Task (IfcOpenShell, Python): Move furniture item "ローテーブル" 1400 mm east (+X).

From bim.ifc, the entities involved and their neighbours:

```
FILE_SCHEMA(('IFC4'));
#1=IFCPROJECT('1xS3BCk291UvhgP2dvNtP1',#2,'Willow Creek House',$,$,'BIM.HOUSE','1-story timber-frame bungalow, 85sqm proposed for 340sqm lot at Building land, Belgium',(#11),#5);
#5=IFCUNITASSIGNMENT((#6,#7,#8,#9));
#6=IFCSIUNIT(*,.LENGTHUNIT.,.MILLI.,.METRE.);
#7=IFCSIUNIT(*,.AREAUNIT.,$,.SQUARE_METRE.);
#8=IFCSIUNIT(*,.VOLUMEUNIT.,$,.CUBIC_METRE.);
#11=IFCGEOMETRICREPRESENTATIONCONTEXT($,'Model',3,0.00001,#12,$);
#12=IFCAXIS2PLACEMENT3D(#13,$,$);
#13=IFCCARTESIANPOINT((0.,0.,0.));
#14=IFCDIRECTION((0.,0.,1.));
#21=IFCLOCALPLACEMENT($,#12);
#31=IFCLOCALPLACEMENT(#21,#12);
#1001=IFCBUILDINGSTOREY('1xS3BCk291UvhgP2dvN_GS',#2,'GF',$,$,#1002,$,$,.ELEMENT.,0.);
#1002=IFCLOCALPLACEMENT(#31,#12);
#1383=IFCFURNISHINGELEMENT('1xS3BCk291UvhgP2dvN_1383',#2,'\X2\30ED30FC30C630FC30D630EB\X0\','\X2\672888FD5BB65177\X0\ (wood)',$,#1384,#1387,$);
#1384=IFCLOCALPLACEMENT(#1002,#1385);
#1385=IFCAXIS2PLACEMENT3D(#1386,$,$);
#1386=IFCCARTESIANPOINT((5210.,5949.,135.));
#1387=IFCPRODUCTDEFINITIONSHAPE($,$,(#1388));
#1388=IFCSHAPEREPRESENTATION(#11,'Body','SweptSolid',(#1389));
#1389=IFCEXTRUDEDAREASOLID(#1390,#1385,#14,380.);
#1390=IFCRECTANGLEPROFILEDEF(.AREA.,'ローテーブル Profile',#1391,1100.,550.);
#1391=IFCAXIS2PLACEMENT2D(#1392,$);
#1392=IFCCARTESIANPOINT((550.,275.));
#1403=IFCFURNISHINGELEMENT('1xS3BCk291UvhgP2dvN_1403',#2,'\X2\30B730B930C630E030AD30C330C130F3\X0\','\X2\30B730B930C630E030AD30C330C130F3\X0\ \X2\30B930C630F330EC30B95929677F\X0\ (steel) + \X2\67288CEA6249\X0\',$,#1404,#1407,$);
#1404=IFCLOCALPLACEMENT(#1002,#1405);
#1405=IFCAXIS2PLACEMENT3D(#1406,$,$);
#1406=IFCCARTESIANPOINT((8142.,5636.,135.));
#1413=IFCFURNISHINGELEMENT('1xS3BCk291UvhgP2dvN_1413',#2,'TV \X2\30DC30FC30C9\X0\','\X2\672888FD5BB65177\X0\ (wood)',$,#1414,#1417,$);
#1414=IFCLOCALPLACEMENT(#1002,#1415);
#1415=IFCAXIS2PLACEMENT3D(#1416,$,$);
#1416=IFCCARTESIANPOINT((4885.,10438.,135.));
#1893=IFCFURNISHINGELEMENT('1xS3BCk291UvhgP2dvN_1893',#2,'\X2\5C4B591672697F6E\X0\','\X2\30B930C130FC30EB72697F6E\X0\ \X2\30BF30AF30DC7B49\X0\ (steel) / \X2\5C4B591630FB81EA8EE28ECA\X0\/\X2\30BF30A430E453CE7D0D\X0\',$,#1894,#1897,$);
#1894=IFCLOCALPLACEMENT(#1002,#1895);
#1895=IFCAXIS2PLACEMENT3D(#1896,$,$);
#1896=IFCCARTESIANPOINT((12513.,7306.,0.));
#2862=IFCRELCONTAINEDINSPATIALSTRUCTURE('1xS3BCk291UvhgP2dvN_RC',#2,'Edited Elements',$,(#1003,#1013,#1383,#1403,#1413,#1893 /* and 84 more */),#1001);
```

```python
import ifcopenshell
import ifcopenshell.api.geometry
import ifcopenshell.util.placement
import ifcopenshell.util.unit

model = ifcopenshell.open("bim.ifc")
unit_scale = ifcopenshell.util.unit.calculate_unit_scale(model)

item = model.by_guid("1xS3BCk291UvhgP2dvN_1383")
matrix = ifcopenshell.util.placement.get_local_placement(item.ObjectPlacement)
matrix[0, 3] += 1.4 / unit_scale
ifcopenshell.api.geometry.edit_object_placement(model, product=item, matrix=matrix, is_si=False)

print(ifcopenshell.util.placement.get_local_placement(item.ObjectPlacement).round(3) + 0.0)

model.write("bim_v2.ifc")
```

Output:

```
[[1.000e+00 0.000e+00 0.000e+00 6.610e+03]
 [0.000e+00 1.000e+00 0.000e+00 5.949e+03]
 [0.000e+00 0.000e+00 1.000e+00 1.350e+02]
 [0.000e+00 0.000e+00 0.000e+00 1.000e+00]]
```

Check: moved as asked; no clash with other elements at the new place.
